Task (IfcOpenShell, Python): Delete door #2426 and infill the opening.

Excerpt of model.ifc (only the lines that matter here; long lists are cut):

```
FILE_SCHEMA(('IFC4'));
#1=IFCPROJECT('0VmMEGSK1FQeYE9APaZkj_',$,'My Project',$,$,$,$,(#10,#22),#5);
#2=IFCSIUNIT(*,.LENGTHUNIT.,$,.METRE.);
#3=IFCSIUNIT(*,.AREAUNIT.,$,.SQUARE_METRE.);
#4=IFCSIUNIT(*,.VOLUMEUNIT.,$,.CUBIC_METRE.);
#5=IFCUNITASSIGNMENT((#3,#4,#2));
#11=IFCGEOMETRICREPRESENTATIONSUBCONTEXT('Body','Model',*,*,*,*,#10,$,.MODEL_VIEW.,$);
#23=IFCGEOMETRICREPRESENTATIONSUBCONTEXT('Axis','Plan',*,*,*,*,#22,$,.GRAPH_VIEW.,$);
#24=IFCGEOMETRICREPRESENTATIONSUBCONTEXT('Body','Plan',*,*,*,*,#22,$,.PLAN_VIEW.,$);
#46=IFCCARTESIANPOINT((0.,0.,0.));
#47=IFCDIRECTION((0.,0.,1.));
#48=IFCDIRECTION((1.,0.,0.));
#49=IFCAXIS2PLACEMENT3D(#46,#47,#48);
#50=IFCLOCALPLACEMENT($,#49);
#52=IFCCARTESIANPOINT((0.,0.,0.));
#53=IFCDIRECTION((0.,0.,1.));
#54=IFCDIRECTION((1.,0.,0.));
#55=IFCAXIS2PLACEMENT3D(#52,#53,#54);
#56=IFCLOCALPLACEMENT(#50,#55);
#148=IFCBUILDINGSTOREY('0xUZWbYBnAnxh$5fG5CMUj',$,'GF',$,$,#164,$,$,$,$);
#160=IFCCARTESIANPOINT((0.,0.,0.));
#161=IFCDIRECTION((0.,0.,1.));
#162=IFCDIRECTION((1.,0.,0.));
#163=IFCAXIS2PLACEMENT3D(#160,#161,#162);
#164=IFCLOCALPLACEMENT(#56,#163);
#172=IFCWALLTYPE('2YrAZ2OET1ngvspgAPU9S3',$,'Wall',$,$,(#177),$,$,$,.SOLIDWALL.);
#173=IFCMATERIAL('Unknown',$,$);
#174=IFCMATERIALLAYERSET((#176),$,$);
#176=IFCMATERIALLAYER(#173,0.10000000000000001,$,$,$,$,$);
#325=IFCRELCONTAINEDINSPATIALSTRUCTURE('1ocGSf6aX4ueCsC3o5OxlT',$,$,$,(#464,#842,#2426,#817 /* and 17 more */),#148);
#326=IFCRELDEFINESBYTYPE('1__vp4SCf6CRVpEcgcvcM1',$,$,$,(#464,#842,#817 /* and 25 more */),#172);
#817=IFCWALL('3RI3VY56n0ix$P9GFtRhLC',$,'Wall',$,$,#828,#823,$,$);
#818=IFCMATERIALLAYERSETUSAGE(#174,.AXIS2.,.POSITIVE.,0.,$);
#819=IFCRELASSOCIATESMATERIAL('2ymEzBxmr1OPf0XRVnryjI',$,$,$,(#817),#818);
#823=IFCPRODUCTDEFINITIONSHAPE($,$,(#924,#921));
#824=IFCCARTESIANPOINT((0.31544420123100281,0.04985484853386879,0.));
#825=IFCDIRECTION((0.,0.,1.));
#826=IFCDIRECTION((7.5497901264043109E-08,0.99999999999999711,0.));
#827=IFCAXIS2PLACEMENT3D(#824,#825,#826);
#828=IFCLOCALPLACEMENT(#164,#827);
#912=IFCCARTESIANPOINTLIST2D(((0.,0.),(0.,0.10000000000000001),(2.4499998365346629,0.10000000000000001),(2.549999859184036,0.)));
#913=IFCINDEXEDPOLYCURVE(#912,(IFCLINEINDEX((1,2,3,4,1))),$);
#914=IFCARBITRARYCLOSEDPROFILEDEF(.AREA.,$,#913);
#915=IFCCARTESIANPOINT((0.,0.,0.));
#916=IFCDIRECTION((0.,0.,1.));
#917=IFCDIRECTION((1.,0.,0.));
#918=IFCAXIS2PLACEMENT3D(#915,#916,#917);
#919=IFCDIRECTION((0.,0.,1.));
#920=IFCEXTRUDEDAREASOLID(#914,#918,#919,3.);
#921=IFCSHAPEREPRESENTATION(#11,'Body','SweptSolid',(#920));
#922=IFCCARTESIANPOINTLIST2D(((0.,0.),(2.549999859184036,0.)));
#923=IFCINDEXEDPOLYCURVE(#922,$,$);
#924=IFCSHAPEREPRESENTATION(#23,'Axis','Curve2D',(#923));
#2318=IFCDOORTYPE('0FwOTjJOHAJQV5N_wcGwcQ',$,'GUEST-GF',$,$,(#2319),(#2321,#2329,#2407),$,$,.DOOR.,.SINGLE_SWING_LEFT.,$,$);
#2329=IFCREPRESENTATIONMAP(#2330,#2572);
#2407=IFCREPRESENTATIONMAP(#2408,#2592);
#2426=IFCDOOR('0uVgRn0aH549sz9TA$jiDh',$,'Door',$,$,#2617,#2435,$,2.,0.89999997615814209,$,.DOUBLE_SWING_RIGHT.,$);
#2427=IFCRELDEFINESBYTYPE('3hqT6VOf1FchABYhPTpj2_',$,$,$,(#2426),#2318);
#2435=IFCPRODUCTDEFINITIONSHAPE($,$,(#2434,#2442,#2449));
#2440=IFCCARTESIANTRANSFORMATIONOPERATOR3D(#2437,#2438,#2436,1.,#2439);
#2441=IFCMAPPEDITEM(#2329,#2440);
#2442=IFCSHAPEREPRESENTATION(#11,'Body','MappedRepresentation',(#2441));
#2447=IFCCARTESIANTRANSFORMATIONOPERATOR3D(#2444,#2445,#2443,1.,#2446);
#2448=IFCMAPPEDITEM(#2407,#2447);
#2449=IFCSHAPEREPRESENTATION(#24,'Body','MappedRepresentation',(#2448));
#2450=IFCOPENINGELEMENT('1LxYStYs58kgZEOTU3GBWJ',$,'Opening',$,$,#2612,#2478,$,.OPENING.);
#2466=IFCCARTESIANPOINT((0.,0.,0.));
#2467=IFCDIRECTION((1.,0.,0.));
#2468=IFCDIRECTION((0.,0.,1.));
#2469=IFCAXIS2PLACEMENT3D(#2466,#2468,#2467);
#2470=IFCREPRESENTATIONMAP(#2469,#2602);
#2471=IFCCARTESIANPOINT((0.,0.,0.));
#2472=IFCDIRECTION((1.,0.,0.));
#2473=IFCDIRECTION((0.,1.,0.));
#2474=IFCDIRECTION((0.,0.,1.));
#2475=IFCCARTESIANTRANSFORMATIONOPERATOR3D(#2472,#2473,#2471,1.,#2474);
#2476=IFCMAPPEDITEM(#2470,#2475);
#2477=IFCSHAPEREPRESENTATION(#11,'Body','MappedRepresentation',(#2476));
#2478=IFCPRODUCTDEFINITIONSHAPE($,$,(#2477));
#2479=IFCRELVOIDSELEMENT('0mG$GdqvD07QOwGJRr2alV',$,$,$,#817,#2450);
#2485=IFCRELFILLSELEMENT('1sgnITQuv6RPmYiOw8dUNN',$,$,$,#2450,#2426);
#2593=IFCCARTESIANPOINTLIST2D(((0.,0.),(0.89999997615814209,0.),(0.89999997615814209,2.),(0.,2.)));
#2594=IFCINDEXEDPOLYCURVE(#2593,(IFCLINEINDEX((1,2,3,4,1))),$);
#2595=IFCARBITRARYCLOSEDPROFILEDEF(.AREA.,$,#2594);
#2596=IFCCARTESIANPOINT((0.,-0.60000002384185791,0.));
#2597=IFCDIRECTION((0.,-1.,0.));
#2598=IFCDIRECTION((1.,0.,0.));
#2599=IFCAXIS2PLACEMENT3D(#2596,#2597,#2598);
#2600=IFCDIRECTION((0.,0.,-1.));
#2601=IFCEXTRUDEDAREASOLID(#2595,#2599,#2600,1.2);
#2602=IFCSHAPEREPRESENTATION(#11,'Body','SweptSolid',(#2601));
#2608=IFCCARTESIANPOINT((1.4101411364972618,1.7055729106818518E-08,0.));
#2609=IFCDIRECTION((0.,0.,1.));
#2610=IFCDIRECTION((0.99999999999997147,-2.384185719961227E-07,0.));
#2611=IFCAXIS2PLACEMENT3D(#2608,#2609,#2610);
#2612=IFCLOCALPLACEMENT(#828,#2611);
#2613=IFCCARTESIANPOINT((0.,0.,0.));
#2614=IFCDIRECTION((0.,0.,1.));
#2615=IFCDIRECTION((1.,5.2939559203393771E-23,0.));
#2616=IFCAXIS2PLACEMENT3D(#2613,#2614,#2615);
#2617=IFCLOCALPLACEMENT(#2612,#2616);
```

```python
import ifcopenshell
import ifcopenshell.api.feature
import ifcopenshell.api.root
import ifcopenshell.geom
import ifcopenshell.util.shape

model = ifcopenshell.open("model.ifc")
settings = ifcopenshell.geom.settings()


def volume(element):
    """Net volume in cubic metres, openings subtracted."""
    shape = ifcopenshell.geom.create_shape(settings, element)
    return ifcopenshell.util.shape.get_volume(shape.geometry)


door = model.by_guid("0uVgRn0aH549sz9TA$jiDh")
opening = door.FillsVoids[0].RelatingOpeningElement
wall = opening.VoidsElements[0].RelatingBuildingElement
before = volume(wall)

ifcopenshell.api.root.remove_product(model, product=door)
ifcopenshell.api.feature.remove_feature(model, feature=opening)

after = volume(wall)

print(f"wall volume {before:.3f} -> {after:.3f} m3")

model.write("model_updated.ifc")
```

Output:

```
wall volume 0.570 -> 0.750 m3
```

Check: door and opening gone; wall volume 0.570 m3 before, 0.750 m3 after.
